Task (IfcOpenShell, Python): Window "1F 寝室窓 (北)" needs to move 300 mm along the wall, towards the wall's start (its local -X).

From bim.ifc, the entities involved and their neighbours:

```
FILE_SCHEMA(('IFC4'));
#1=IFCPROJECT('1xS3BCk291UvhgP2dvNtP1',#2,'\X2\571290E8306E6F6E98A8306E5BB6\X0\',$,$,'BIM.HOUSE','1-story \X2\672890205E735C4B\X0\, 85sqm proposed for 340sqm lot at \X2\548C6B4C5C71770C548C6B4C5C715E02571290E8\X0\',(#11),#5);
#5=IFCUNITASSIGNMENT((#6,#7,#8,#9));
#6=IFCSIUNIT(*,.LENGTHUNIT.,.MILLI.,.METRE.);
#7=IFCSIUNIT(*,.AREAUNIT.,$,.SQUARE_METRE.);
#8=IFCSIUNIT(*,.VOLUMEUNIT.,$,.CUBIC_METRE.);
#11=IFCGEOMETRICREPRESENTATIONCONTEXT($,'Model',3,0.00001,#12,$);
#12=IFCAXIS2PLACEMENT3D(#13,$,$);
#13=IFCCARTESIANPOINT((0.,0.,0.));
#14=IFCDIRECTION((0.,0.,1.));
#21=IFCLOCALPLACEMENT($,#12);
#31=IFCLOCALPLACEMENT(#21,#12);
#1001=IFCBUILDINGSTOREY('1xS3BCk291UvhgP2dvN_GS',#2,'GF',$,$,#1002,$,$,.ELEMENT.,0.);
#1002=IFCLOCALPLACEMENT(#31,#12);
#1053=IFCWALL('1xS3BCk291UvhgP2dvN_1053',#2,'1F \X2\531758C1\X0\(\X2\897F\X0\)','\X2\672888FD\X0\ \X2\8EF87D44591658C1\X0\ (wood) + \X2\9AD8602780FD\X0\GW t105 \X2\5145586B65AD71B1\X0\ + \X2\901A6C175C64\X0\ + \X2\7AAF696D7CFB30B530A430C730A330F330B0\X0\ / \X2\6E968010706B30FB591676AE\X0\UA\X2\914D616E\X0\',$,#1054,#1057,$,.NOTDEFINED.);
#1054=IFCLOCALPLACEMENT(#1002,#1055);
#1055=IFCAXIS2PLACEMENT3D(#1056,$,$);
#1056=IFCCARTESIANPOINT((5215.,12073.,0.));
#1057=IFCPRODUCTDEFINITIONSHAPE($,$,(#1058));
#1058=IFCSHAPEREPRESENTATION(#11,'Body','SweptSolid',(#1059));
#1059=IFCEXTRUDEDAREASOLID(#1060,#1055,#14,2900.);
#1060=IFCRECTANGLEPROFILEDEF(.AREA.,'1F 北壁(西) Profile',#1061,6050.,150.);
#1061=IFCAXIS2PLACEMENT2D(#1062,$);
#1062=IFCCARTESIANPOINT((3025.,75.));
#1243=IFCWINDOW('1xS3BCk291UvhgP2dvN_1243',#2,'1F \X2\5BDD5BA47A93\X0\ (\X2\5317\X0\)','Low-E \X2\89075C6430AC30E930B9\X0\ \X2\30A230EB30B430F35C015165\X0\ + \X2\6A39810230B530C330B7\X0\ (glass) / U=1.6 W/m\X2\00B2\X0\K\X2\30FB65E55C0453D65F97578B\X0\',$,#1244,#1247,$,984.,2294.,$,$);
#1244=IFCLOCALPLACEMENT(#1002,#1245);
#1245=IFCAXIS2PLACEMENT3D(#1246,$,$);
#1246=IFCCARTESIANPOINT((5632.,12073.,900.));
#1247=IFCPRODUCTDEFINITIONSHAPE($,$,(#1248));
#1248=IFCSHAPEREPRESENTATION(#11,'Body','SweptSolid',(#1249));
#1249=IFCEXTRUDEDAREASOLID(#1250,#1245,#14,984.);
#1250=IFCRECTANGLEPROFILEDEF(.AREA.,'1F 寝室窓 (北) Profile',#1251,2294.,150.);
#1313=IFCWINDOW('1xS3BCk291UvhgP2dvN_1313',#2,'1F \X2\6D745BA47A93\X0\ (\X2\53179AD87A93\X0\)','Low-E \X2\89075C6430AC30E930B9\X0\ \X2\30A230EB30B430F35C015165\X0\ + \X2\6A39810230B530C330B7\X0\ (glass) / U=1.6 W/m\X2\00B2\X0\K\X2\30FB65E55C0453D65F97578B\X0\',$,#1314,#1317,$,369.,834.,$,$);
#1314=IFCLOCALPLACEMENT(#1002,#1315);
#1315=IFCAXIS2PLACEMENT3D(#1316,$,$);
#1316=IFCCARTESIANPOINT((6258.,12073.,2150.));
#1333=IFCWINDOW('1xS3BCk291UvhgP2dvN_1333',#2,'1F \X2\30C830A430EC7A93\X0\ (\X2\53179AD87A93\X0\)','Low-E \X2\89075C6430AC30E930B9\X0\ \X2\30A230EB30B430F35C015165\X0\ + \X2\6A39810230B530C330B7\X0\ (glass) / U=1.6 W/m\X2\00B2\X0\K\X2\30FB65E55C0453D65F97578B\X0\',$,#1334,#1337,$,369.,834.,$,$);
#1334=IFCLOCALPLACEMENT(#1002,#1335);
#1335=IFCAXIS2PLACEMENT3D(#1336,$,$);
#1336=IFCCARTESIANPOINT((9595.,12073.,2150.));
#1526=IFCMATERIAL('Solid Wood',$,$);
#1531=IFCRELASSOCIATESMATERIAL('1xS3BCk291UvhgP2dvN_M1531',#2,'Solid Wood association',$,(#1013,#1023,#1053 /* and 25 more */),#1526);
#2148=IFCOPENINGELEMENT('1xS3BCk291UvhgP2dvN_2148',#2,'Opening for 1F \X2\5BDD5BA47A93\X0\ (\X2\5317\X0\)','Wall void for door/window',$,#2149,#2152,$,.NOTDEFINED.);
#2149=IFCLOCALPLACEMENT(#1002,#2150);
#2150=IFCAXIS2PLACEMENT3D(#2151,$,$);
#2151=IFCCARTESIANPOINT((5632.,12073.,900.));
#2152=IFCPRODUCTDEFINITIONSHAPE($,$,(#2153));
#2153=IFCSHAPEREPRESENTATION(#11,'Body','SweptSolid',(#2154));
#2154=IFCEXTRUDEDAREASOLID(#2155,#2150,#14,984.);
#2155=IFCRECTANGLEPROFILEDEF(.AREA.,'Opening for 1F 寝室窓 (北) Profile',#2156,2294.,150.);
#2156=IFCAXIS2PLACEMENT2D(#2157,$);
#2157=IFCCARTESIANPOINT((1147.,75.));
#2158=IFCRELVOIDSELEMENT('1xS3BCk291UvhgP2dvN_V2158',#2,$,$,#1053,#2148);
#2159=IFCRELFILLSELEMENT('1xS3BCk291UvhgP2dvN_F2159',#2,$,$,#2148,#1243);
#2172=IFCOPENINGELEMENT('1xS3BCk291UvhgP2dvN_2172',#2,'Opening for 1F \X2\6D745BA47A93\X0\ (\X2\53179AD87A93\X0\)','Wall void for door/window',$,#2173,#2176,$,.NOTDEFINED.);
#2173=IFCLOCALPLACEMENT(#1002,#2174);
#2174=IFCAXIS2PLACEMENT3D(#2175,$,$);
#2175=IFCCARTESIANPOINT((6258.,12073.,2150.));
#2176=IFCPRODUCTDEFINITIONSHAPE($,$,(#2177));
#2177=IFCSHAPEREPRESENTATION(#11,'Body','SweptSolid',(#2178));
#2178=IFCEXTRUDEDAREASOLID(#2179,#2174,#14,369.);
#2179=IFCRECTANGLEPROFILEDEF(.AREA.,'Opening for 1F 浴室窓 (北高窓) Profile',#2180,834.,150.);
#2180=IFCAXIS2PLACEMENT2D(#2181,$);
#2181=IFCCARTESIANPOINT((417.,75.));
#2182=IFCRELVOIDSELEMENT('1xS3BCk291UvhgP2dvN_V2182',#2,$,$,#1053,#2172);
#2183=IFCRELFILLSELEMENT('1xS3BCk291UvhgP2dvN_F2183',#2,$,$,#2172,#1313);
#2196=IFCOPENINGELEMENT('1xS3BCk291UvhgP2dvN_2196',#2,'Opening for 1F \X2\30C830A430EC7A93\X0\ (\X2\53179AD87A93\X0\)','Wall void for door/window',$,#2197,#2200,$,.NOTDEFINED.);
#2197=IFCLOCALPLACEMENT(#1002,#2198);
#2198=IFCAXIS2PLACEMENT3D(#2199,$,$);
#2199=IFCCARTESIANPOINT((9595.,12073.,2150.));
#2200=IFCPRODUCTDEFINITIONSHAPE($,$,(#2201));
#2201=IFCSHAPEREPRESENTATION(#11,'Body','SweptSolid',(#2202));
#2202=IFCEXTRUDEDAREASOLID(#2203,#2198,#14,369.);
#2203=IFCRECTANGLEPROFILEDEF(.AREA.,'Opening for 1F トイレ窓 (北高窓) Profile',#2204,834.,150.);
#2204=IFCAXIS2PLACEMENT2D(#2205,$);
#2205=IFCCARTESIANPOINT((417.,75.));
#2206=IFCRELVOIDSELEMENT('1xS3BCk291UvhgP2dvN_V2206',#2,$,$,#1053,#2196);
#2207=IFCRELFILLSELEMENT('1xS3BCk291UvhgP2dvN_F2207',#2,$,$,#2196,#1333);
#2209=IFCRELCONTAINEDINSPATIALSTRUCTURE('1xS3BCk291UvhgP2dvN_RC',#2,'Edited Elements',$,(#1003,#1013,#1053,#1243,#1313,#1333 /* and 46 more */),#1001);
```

```python
import ifcopenshell
import ifcopenshell.api.geometry
import ifcopenshell.util.placement

model = ifcopenshell.open("bim.ifc")

window = model.by_guid("1xS3BCk291UvhgP2dvN_1243")
opening = window.FillsVoids[0].RelatingOpeningElement
wall = opening.VoidsElements[0].RelatingBuildingElement

wall_matrix = ifcopenshell.util.placement.get_local_placement(wall.ObjectPlacement)
shift = wall_matrix[:3, 0] * -300.0
before = ifcopenshell.util.placement.get_local_placement(window.ObjectPlacement)[:3, 3].copy()

# The window is not placed relative to its opening, so move both.
for product in (opening, window):
    matrix = ifcopenshell.util.placement.get_local_placement(product.ObjectPlacement)
    matrix[:3, 3] += shift
    ifcopenshell.api.geometry.edit_object_placement(model, product=product, matrix=matrix, is_si=False)

after = ifcopenshell.util.placement.get_local_placement(window.ObjectPlacement)[:3, 3]
print("window moved by", (after - before).round(3) + 0.0)

model.write("bim_updated.ifc")
```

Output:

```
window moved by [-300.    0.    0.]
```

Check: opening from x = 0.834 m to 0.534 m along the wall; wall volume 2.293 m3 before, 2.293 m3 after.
